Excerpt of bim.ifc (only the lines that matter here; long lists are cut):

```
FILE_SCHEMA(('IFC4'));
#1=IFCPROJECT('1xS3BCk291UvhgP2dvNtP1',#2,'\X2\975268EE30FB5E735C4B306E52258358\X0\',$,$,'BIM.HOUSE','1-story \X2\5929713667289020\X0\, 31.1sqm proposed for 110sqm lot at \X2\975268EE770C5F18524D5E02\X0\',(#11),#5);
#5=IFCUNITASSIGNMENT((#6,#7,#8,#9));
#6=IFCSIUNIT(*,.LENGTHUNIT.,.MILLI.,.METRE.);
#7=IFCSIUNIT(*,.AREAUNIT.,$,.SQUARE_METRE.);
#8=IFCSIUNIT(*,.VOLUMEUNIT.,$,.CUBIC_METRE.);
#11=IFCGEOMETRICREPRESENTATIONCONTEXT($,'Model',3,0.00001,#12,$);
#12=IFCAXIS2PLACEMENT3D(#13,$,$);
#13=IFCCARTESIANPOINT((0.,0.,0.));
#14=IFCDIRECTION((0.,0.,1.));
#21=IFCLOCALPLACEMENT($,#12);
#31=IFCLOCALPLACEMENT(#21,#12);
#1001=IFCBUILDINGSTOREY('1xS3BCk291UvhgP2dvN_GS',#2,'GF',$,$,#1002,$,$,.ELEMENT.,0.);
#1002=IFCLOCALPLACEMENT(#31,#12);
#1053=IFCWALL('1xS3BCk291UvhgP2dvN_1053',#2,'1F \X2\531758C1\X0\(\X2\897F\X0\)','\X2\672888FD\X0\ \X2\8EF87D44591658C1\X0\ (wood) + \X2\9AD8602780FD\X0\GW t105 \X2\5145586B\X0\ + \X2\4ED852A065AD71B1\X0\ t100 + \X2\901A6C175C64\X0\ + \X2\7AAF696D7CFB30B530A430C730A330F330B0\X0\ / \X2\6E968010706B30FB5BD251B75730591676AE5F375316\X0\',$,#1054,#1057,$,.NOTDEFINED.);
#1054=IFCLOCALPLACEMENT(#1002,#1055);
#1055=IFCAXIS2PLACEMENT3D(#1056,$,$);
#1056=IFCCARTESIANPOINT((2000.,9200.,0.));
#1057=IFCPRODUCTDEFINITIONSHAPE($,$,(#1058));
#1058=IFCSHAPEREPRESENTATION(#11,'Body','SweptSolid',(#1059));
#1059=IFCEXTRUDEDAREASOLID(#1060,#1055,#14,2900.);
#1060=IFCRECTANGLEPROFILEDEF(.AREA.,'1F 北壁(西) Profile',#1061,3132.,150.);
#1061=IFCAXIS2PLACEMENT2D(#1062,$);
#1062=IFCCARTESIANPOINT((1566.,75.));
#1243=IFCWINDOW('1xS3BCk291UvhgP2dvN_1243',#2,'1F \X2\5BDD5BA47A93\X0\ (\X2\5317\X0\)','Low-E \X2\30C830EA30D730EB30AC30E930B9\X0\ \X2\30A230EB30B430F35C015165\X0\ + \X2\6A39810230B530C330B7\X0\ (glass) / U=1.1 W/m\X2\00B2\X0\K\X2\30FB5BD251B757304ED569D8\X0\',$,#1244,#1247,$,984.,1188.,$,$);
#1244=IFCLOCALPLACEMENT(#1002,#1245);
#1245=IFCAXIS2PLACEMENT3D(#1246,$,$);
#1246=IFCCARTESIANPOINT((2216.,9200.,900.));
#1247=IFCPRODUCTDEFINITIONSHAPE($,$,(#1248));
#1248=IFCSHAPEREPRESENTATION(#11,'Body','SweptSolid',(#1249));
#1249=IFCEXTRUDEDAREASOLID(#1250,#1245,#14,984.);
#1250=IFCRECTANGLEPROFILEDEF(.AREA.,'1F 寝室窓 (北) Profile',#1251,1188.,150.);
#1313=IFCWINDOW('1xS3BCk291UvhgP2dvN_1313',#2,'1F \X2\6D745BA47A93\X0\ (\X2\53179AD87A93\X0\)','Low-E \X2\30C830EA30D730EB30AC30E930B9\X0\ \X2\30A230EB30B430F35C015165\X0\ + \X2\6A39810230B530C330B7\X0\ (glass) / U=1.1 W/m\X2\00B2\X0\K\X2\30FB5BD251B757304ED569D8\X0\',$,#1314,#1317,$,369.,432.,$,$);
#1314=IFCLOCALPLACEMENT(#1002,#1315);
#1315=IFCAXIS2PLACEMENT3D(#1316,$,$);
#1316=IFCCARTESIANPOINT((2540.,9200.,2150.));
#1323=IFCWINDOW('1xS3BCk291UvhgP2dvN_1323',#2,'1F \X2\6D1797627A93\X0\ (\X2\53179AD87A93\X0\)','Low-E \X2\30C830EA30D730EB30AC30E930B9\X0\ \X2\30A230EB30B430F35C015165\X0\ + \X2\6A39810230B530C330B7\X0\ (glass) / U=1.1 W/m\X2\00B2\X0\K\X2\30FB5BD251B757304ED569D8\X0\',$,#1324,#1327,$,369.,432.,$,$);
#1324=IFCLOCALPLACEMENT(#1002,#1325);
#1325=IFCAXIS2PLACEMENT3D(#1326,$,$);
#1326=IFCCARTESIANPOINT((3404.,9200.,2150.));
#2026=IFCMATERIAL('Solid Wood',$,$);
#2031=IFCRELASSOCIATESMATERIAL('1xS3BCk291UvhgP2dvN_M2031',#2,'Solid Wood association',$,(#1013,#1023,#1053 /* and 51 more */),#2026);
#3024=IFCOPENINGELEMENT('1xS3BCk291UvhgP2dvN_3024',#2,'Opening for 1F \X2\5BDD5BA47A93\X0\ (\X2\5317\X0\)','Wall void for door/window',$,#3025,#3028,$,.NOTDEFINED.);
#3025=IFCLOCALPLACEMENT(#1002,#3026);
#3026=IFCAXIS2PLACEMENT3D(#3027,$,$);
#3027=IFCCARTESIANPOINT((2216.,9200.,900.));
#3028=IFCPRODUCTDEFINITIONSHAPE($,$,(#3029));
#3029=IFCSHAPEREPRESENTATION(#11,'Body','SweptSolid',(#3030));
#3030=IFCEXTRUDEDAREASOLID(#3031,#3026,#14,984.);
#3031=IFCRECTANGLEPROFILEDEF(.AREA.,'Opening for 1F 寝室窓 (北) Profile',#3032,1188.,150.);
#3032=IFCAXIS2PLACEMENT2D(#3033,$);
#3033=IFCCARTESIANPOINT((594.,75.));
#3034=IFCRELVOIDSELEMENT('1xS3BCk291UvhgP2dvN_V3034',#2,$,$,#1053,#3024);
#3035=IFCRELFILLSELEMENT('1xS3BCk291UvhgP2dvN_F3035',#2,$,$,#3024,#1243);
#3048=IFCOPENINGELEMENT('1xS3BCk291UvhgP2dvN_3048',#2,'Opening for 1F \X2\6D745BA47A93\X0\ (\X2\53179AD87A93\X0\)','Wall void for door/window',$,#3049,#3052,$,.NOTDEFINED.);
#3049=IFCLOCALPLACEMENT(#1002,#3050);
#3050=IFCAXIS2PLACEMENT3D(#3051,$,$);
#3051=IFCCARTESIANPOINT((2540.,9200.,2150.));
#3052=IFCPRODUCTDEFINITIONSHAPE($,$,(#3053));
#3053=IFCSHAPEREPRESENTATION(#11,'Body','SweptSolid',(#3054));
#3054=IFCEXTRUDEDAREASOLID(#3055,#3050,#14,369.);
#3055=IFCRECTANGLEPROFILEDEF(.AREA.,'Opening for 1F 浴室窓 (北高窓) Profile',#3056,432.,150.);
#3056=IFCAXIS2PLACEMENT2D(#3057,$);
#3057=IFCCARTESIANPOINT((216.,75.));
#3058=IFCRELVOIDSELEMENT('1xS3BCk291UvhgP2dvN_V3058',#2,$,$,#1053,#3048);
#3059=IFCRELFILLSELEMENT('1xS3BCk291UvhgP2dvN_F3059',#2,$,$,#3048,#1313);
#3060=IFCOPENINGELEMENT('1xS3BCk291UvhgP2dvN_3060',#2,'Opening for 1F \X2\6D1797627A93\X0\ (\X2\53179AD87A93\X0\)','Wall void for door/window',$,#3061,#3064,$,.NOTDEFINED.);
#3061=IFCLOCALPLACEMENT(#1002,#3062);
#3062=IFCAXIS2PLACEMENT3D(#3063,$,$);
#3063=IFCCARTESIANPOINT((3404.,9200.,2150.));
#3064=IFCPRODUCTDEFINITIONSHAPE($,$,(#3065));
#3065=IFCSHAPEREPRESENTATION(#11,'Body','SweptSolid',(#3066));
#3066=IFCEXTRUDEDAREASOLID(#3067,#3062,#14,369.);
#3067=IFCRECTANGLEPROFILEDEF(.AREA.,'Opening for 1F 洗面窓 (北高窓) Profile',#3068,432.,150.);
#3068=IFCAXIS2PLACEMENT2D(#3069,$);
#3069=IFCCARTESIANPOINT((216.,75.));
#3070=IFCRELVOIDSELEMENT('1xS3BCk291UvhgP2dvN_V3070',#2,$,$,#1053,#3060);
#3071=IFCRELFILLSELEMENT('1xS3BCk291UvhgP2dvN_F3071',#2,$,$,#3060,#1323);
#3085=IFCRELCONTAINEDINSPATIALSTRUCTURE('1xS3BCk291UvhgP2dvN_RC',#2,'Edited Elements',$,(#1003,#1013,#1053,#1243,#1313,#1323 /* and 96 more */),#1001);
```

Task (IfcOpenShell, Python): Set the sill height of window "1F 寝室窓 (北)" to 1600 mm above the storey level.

```python
import numpy as np
import ifcopenshell
import ifcopenshell.api.geometry
import ifcopenshell.geom
import ifcopenshell.util.element
import ifcopenshell.util.placement
import ifcopenshell.util.shape
import ifcopenshell.util.unit

model = ifcopenshell.open("bim.ifc")
unit_scale = ifcopenshell.util.unit.calculate_unit_scale(model)

window = model.by_guid("1xS3BCk291UvhgP2dvN_1243")
opening = window.FillsVoids[0].RelatingOpeningElement
storey = ifcopenshell.util.element.get_container(window, ifc_class="IfcBuildingStorey")
level = ifcopenshell.util.placement.get_local_placement(storey.ObjectPlacement)[2, 3]

# The opening's origin need not be at the sill, so measure its lowest point.
shape = ifcopenshell.geom.create_shape(ifcopenshell.geom.settings(), opening)
bottom = ifcopenshell.util.shape.get_shape_bottom_elevation(shape, shape.geometry) / unit_scale
dz = level + 1.6 / unit_scale - bottom

shift = np.array([0.0, 0.0, dz])
# The window is not placed relative to its opening, so move both.
for product in (opening, window):
    matrix = ifcopenshell.util.placement.get_local_placement(product.ObjectPlacement)
    matrix[:3, 3] += shift
    ifcopenshell.api.geometry.edit_object_placement(model, product=product, matrix=matrix, is_si=False)

print(f"moved by {dz * unit_scale:+.3f} m")

model.write("bim_updated.ifc")
```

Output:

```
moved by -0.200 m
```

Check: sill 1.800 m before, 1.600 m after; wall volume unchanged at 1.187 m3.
